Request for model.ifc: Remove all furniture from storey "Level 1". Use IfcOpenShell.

First a look at what the model holds.

```python
import ifcopenshell
import ifcopenshell.util.element

model = ifcopenshell.open("model.ifc")
print(model.schema)
storey = next(s for s in model.by_type("IfcBuildingStorey") if s.Name == "Level 1")
furniture = [e for e in ifcopenshell.util.element.get_decomposition(storey) if e.is_a("IfcFurnishingElement")]
seen = {}
for e in furniture:
    element_type = ifcopenshell.util.element.get_type(e)
    name = element_type.Name if element_type not in (None, e) else None
    seen[name] = seen.get(name, 0) + 1
for name, count in sorted(seen.items(), key=str):
    print(count, "x", name)
```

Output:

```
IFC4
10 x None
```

```python
import ifcopenshell
import ifcopenshell.api.root
import ifcopenshell.util.element

model = ifcopenshell.open("model.ifc")

storey = next(s for s in model.by_type("IfcBuildingStorey") if s.Name == "Level 1")
furniture = [e for e in ifcopenshell.util.element.get_decomposition(storey) if e.is_a("IfcFurnishingElement")]

for e in furniture:
    ifcopenshell.api.root.remove_product(model, product=e)
print(len(furniture), "removed")

model.write("model_v2.ifc")
```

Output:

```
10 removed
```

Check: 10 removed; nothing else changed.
